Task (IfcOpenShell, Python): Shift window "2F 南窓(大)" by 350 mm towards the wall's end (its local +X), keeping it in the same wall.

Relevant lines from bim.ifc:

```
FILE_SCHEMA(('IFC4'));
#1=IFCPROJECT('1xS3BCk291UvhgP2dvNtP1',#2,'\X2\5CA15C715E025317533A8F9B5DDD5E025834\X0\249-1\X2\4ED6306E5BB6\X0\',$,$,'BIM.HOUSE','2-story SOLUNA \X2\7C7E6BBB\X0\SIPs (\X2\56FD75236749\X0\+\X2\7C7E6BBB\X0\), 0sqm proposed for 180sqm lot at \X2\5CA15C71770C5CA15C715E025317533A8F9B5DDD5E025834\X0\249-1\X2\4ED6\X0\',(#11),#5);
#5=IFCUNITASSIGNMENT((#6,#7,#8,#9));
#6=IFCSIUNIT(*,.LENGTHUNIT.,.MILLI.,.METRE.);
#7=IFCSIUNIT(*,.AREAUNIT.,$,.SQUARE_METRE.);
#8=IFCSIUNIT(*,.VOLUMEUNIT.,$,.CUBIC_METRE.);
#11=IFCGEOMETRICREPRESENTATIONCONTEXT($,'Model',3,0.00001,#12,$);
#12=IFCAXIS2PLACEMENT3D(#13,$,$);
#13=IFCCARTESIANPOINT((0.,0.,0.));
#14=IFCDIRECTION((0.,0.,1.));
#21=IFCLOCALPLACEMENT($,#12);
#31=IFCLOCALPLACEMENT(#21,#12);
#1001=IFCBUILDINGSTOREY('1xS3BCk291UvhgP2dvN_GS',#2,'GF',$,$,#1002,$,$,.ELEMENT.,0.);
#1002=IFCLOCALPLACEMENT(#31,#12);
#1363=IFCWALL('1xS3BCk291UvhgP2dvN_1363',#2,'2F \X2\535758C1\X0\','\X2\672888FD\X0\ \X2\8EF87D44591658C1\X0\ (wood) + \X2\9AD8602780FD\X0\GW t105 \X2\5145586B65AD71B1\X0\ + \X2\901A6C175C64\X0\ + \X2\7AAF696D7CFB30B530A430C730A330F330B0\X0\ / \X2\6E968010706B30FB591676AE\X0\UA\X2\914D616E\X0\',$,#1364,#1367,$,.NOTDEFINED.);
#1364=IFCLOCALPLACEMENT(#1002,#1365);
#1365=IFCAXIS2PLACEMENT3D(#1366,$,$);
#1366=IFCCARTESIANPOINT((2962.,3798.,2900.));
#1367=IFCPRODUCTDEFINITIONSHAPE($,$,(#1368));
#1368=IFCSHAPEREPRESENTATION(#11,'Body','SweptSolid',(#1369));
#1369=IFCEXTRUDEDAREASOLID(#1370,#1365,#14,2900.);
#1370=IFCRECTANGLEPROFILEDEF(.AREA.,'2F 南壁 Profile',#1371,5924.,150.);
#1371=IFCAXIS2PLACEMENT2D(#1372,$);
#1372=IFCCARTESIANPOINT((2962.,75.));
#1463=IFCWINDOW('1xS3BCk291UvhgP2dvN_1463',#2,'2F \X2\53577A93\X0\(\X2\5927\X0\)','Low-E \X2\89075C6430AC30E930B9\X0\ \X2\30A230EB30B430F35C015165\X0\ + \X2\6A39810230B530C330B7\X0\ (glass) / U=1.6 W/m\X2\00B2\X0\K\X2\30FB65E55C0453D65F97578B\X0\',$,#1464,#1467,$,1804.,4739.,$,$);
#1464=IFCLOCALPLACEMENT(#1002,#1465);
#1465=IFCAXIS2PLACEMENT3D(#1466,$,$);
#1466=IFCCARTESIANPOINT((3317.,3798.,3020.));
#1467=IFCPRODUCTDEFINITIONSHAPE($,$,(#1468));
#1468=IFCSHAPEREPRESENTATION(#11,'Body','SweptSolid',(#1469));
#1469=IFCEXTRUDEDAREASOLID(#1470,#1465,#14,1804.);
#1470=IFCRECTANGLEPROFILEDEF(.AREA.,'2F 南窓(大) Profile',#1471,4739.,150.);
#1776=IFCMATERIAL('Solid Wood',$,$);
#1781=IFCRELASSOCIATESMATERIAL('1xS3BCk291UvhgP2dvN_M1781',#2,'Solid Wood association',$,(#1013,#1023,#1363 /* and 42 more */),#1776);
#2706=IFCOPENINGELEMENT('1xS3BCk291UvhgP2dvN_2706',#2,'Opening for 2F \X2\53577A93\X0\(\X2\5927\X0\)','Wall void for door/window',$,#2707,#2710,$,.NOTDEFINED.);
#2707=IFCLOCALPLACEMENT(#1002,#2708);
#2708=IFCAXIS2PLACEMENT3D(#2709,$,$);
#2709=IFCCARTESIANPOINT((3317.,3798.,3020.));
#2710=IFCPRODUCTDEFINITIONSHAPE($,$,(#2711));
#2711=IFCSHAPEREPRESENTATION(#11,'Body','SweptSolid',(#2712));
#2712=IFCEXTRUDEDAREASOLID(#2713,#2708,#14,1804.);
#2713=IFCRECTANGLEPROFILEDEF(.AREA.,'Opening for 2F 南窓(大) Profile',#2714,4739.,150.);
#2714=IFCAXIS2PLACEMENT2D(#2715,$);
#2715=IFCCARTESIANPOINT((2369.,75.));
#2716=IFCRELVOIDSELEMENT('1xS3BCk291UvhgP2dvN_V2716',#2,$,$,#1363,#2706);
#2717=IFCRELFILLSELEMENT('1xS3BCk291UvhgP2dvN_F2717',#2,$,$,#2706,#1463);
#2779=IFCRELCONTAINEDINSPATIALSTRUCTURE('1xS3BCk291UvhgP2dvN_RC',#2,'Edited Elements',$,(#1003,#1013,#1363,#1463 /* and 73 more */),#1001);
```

```python
import ifcopenshell
import ifcopenshell.api.geometry
import ifcopenshell.util.placement
import ifcopenshell.util.unit

model = ifcopenshell.open("bim.ifc")
unit_scale = ifcopenshell.util.unit.calculate_unit_scale(model)

window = model.by_guid("1xS3BCk291UvhgP2dvN_1463")
opening = window.FillsVoids[0].RelatingOpeningElement
wall = opening.VoidsElements[0].RelatingBuildingElement

wall_matrix = ifcopenshell.util.placement.get_local_placement(wall.ObjectPlacement)
shift = wall_matrix[:3, 0] * 0.35 / unit_scale
before = ifcopenshell.util.placement.get_local_placement(window.ObjectPlacement)[:3, 3].copy()

# The window is not placed relative to its opening, so move both.
for product in (opening, window):
    matrix = ifcopenshell.util.placement.get_local_placement(product.ObjectPlacement)
    matrix[:3, 3] += shift
    ifcopenshell.api.geometry.edit_object_placement(model, product=product, matrix=matrix, is_si=False)

after = ifcopenshell.util.placement.get_local_placement(window.ObjectPlacement)[:3, 3]
print("window moved by", (after - before).round(3) + 0.0)

model.write("bim-out.ifc")
```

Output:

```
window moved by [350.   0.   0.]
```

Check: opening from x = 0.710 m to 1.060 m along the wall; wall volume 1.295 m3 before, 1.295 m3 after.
